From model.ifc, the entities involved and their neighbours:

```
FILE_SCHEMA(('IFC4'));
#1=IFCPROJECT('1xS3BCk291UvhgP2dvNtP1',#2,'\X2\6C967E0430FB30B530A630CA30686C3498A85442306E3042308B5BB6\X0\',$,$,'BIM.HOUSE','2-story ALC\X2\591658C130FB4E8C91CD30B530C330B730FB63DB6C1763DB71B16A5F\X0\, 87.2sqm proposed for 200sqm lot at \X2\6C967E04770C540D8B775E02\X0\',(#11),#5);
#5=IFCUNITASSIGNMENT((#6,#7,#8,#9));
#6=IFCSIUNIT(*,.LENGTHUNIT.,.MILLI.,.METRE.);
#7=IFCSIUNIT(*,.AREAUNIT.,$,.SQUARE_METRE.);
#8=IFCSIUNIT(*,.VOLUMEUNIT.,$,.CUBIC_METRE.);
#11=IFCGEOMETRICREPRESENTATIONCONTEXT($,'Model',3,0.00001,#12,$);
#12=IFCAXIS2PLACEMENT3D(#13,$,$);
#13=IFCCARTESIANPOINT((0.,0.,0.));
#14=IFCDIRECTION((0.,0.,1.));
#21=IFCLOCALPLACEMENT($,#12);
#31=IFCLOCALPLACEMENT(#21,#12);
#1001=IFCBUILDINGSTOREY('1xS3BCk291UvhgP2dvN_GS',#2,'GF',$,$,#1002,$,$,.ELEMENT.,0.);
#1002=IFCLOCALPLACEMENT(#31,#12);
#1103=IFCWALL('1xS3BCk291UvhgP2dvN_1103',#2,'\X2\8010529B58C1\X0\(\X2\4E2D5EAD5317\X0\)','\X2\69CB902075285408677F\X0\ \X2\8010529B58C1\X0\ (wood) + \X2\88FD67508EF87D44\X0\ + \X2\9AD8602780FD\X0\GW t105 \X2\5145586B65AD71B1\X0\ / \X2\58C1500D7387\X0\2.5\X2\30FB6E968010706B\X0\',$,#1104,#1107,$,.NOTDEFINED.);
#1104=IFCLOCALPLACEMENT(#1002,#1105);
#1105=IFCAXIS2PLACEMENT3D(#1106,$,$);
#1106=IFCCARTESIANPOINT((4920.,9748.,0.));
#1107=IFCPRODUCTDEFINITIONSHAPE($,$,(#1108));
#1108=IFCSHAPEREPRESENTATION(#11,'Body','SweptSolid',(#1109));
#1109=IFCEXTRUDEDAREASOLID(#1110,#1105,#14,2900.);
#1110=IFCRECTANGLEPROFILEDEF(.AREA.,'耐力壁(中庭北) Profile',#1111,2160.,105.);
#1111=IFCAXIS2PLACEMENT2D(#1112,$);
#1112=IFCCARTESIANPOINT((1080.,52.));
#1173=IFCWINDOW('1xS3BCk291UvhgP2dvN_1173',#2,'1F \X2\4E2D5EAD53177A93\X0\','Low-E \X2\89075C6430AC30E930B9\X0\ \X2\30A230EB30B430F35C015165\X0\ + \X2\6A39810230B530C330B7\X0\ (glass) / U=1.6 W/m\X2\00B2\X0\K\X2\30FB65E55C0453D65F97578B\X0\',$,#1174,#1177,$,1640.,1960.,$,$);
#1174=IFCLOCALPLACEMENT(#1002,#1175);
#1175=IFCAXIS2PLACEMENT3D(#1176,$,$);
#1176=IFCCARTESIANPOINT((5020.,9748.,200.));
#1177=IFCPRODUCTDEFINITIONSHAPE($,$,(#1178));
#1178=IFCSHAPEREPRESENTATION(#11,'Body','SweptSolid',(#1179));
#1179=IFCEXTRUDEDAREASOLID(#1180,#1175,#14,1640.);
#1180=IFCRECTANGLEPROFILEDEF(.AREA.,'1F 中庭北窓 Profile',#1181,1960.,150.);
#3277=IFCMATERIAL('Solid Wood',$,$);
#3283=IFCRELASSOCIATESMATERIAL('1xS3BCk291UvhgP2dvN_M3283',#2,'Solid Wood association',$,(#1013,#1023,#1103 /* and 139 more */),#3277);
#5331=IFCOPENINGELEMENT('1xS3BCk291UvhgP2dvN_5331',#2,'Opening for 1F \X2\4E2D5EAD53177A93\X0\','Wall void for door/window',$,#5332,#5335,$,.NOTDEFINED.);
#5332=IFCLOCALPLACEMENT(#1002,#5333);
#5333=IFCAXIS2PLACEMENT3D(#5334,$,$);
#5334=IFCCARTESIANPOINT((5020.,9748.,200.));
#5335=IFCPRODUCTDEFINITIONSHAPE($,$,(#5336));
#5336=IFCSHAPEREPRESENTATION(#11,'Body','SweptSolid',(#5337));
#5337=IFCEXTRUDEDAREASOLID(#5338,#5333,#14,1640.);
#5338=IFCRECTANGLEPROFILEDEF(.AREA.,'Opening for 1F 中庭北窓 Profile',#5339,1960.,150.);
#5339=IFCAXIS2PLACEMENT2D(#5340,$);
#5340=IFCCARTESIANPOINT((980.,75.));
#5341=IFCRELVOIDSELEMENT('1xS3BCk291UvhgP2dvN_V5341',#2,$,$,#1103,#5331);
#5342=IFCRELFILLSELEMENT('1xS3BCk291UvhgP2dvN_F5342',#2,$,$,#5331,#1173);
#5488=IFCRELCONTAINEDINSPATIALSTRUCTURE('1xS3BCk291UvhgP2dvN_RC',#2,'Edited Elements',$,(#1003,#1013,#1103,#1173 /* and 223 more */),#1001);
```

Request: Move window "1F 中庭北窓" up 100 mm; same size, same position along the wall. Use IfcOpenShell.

```python
import numpy as np
import ifcopenshell
import ifcopenshell.api.geometry
import ifcopenshell.util.placement
import ifcopenshell.util.unit

model = ifcopenshell.open("model.ifc")
unit_scale = ifcopenshell.util.unit.calculate_unit_scale(model)

window = model.by_id(1173)
opening = window.FillsVoids[0].RelatingOpeningElement
dz = 100.0

shift = np.array([0.0, 0.0, dz])
# The window is not placed relative to its opening, so move both.
for product in (opening, window):
    matrix = ifcopenshell.util.placement.get_local_placement(product.ObjectPlacement)
    matrix[:3, 3] += shift
    ifcopenshell.api.geometry.edit_object_placement(model, product=product, matrix=matrix, is_si=False)

print(f"moved by {dz * unit_scale:+.3f} m")

model.write("model_v2.ifc")
```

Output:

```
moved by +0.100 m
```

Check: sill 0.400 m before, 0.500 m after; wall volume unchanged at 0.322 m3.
